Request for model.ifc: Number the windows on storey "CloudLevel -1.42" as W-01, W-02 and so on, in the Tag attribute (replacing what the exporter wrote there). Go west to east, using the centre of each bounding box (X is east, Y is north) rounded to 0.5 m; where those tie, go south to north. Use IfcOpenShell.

First a look at what the model holds.

```python
import ifcopenshell
import ifcopenshell.util.element
import ifcopenshell.util.placement

model = ifcopenshell.open("model.ifc")
print(model.schema)
storey = next(s for s in model.by_type("IfcBuildingStorey") if s.Name == "CloudLevel -1.42")
windows = [e for e in ifcopenshell.util.element.get_decomposition(storey) if e.is_a("IfcWindow")]
for e in sorted(windows, key=lambda e: e.id()):
    origin = ifcopenshell.util.placement.get_local_placement(e.ObjectPlacement)[:3, 3]
    print(e.id(), e.Tag, e.Name, origin.round(2) + 0.0, sep=" | ")
```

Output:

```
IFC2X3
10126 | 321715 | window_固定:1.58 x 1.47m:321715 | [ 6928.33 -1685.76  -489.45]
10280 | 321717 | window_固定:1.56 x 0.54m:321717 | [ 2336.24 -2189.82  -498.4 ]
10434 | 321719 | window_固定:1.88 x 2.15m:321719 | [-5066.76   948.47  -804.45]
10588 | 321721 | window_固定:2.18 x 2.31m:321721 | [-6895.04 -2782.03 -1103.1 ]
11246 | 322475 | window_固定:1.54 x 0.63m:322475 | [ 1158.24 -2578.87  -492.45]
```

```python
import ifcopenshell
import ifcopenshell.geom
import ifcopenshell.util.element
import ifcopenshell.util.shape

model = ifcopenshell.open("model.ifc")
settings = ifcopenshell.geom.settings()
settings.set("use-world-coords", True)


def centre(element):
    shape = ifcopenshell.geom.create_shape(settings, element)
    return ifcopenshell.util.shape.get_bbox_centroid(shape.geometry)


storey = next(s for s in model.by_type("IfcBuildingStorey") if s.Name == "CloudLevel -1.42")
windows = [e for e in ifcopenshell.util.element.get_decomposition(storey) if e.is_a("IfcWindow")]

# Insertion points can sit at a corner or the storey origin, so sort by the geometry (in metres).
centres = {e: centre(e) for e in windows}
windows.sort(key=lambda e: (round(centres[e][0] / 0.5), centres[e][1]))

for i, e in enumerate(windows, start=1):
    number = f"W-{i:02d}"
    e.Tag = number
    print(e.id(), number)

model.write("model-out.ifc")
```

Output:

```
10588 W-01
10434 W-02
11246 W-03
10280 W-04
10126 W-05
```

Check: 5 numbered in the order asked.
